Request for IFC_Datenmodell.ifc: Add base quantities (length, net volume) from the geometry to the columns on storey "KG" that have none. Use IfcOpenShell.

First a look at what the model holds.

```python
import ifcopenshell
import ifcopenshell.util.element
import ifcopenshell.util.unit

model = ifcopenshell.open("IFC_Datenmodell.ifc")
print(model.schema)
for unit_type in ("LENGTHUNIT", "AREAUNIT", "VOLUMEUNIT"):
    print(unit_type, ifcopenshell.util.unit.calculate_unit_scale(model, unit_type))
storey = next(s for s in model.by_type("IfcBuildingStorey") if s.Name == "KG")
columns = [e for e in ifcopenshell.util.element.get_decomposition(storey) if e.is_a("IfcColumn")]
for e in sorted(columns, key=lambda e: e.id()):
    print(e.id(), e.is_a(), e.Name, list(ifcopenshell.util.element.get_psets(e, qtos_only=True)), sep=" | ")
```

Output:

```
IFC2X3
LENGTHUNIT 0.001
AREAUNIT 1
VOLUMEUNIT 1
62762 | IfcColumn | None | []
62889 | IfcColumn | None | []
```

```python
import ifcopenshell
import ifcopenshell.api.pset
import ifcopenshell.geom
import ifcopenshell.util.element
import ifcopenshell.util.shape
import ifcopenshell.util.unit

model = ifcopenshell.open("IFC_Datenmodell.ifc")
unit_scale = ifcopenshell.util.unit.calculate_unit_scale(model)
volume_scale = ifcopenshell.util.unit.calculate_unit_scale(model, "VOLUMEUNIT")
settings = ifcopenshell.geom.settings()

storey = next(s for s in model.by_type("IfcBuildingStorey") if s.Name == "KG")
columns = [e for e in ifcopenshell.util.element.get_decomposition(storey) if e.is_a("IfcColumn")]

for e in sorted(columns, key=lambda e: e.id()):
    if ifcopenshell.util.element.get_psets(e, qtos_only=True, should_inherit=False):
        continue
    # Geometry comes back in metres, in the element's own axes.
    shape = ifcopenshell.geom.create_shape(settings, e)
    values = {
        "Length": ifcopenshell.util.shape.get_z(shape.geometry) / unit_scale,
        "NetVolume": ifcopenshell.util.shape.get_volume(shape.geometry) / volume_scale,
    }
    qto = ifcopenshell.api.pset.add_qto(model, product=e, name="BaseQuantities")
    ifcopenshell.api.pset.edit_qto(model, qto=qto, properties=values)
    print(e.id(), {k: round(v, 3) for k, v in values.items()})

model.write("IFC_Datenmodell_edited.ifc")
```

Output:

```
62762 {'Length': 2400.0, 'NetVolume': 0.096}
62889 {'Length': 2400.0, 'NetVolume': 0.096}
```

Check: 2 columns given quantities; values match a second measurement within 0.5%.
